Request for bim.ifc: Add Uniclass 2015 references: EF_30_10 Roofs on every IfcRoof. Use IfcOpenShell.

First a look at what the model holds.

```python
import ifcopenshell

model = ifcopenshell.open("bim.ifc")
print(model.schema)
print("classifications:", [c.Name for c in model.by_type("IfcClassification")])
for ifc_class in ("IfcDoor", "IfcRoof", "IfcStair", "IfcWall", "IfcWindow"):
    print(ifc_class, len(model.by_type(ifc_class)))
```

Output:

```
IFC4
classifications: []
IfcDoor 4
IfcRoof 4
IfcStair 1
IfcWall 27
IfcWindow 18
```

```python
import ifcopenshell
import ifcopenshell.api.classification

model = ifcopenshell.open("bim.ifc")

system = ifcopenshell.api.classification.add_classification(model, classification="Uniclass 2015")

codes = {
    "IfcRoof": ("EF_30_10", "Roofs"),
}
for ifc_class, (code, name) in codes.items():
    products = model.by_type(ifc_class)
    ifcopenshell.api.classification.add_reference(
        model, products=products, classification=system, identification=code, name=name
    )
    print(code, len(products))

model.write("bim_edited.ifc")
```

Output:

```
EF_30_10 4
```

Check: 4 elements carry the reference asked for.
